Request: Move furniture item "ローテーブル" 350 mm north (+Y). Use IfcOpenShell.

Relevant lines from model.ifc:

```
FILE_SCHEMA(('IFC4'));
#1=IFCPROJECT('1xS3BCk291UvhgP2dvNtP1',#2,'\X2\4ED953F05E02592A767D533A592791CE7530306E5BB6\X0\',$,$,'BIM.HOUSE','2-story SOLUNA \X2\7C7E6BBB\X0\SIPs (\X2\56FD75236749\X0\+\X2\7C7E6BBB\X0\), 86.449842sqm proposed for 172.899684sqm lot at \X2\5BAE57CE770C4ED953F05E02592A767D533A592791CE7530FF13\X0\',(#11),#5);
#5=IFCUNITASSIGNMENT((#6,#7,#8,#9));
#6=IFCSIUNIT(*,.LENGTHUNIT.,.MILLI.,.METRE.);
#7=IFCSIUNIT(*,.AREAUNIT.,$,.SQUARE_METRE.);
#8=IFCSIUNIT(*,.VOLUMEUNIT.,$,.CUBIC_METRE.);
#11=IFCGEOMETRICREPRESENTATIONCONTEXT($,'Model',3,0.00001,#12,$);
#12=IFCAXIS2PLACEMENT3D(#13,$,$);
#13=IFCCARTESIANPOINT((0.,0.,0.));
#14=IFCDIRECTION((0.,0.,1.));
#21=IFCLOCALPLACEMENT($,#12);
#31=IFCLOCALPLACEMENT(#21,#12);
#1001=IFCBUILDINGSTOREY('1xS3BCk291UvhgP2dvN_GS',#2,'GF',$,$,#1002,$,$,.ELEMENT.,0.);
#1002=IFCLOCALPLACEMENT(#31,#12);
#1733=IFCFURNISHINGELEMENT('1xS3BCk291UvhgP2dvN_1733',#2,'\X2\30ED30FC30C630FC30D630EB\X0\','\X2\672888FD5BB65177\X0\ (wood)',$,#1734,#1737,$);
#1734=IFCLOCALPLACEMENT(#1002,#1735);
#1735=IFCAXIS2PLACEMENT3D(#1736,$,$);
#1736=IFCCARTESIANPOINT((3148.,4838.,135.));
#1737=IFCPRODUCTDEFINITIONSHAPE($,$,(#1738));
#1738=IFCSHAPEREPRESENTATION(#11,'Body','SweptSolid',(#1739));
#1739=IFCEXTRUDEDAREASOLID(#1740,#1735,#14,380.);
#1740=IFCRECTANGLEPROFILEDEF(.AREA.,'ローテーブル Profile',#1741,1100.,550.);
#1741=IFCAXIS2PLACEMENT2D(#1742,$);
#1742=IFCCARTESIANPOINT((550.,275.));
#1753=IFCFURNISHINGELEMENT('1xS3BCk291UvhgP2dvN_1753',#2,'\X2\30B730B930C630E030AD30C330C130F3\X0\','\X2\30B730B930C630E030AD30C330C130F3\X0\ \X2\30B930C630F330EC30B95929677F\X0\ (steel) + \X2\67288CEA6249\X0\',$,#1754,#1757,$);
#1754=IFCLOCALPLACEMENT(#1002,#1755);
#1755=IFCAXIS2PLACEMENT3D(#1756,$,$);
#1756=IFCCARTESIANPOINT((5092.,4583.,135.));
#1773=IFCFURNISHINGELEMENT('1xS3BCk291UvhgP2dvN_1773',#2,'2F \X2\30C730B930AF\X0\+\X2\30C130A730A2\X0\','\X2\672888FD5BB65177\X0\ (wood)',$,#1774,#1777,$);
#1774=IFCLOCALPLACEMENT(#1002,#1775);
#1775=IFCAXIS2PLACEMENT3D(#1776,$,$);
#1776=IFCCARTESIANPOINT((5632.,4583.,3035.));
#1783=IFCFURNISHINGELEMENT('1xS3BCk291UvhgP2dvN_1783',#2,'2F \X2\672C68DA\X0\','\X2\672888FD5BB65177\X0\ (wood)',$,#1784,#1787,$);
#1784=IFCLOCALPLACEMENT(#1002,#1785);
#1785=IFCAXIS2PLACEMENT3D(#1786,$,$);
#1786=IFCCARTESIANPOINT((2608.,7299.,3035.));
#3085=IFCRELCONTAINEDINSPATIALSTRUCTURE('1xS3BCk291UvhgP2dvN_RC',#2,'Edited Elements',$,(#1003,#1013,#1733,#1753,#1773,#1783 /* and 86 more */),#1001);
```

```python
import ifcopenshell
import ifcopenshell.api.geometry
import ifcopenshell.util.placement

model = ifcopenshell.open("model.ifc")

item = model.by_id(1733)
matrix = ifcopenshell.util.placement.get_local_placement(item.ObjectPlacement)
matrix[1, 3] += 350.0
ifcopenshell.api.geometry.edit_object_placement(model, product=item, matrix=matrix, is_si=False)

print(ifcopenshell.util.placement.get_local_placement(item.ObjectPlacement).round(3) + 0.0)

model.write("model_v2.ifc")
```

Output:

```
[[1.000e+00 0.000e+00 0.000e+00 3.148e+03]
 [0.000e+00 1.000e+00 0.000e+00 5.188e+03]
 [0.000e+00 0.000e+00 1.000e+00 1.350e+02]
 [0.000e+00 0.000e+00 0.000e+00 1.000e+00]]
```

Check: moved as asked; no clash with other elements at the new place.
